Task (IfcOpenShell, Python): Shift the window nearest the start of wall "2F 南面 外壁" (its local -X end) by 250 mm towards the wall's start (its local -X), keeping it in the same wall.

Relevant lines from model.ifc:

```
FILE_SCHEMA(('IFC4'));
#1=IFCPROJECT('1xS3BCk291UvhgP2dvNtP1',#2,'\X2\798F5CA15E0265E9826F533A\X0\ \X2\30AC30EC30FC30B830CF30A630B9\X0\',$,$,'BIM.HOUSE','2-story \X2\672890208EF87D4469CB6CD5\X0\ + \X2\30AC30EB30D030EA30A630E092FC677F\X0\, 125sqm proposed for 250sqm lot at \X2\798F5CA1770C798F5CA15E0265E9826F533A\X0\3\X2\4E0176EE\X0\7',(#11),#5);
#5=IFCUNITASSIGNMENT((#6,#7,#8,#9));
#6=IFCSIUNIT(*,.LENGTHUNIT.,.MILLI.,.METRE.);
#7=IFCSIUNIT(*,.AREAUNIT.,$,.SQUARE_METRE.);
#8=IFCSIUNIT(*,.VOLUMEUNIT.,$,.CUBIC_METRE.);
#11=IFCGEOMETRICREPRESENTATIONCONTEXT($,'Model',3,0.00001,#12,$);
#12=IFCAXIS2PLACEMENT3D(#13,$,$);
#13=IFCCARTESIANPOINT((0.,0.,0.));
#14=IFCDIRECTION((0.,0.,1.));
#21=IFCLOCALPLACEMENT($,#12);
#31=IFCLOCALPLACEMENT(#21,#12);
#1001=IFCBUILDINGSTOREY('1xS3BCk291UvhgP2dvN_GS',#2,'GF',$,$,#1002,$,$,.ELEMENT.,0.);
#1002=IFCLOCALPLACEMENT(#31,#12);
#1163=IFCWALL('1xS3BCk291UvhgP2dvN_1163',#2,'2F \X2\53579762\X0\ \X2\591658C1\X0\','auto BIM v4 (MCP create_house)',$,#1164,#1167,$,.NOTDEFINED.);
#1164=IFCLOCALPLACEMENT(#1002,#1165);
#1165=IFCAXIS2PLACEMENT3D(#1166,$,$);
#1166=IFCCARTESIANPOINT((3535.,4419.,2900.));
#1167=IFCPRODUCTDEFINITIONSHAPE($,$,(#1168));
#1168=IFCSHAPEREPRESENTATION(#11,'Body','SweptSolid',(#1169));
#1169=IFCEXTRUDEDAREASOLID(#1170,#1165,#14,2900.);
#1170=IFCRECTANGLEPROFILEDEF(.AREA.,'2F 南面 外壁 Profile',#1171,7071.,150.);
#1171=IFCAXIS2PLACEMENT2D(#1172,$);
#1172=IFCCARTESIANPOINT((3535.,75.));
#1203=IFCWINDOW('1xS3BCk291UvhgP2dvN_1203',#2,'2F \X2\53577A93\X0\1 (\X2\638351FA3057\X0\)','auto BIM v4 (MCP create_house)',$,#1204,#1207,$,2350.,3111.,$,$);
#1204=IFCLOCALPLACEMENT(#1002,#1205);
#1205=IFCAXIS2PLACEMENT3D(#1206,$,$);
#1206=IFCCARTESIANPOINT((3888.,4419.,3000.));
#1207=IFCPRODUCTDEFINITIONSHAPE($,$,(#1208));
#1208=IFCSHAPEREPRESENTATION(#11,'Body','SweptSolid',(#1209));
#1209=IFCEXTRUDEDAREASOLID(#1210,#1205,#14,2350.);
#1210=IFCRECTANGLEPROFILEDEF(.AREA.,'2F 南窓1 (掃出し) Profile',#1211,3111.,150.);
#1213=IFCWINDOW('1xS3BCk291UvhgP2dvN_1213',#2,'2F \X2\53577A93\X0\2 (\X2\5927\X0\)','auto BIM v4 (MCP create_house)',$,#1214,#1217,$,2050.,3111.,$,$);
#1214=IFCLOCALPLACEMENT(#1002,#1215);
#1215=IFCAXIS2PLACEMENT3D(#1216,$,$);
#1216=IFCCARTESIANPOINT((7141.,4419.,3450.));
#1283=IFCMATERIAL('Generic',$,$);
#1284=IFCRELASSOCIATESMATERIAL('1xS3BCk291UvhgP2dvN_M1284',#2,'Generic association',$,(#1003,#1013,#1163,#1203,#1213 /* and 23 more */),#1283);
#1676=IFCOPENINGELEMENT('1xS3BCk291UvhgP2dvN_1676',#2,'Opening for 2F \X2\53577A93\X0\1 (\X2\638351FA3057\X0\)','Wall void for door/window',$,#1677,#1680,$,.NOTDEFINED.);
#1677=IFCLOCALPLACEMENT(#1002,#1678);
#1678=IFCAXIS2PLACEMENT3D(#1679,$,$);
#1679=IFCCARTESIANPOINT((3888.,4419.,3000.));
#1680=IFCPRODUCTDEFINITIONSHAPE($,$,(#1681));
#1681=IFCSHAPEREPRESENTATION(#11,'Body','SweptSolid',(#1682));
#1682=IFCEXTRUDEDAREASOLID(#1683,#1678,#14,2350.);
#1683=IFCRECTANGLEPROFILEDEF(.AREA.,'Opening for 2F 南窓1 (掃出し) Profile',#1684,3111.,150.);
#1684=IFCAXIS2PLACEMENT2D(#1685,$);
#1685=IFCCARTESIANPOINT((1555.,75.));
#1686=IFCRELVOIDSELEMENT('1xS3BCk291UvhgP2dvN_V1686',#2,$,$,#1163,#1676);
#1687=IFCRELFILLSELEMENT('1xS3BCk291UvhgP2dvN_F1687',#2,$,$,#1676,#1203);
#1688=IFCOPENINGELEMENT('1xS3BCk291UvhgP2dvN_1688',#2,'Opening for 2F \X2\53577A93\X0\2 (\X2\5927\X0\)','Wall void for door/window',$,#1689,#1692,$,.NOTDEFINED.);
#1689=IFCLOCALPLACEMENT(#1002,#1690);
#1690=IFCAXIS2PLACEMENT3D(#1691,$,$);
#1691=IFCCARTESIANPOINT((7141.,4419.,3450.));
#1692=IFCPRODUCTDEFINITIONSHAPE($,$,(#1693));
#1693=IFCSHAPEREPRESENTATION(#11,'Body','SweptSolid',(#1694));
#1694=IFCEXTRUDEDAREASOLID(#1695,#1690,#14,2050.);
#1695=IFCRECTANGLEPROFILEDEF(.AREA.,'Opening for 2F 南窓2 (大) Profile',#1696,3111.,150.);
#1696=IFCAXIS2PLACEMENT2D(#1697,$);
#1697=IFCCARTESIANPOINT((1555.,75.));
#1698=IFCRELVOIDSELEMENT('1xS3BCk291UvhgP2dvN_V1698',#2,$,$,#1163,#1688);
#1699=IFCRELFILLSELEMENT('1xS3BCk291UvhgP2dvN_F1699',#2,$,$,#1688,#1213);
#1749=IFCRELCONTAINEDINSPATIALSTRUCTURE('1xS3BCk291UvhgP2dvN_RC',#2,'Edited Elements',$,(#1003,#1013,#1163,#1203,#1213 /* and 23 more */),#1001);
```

```python
import ifcopenshell
import ifcopenshell.api.geometry
import ifcopenshell.util.placement
import ifcopenshell.util.unit

model = ifcopenshell.open("model.ifc")
unit_scale = ifcopenshell.util.unit.calculate_unit_scale(model)

window = model.by_guid("1xS3BCk291UvhgP2dvN_1203")
opening = window.FillsVoids[0].RelatingOpeningElement
wall = opening.VoidsElements[0].RelatingBuildingElement

wall_matrix = ifcopenshell.util.placement.get_local_placement(wall.ObjectPlacement)
shift = wall_matrix[:3, 0] * -0.25 / unit_scale
before = ifcopenshell.util.placement.get_local_placement(window.ObjectPlacement)[:3, 3].copy()

# The window is not placed relative to its opening, so move both.
for product in (opening, window):
    matrix = ifcopenshell.util.placement.get_local_placement(product.ObjectPlacement)
    matrix[:3, 3] += shift
    ifcopenshell.api.geometry.edit_object_placement(model, product=product, matrix=matrix, is_si=False)

after = ifcopenshell.util.placement.get_local_placement(window.ObjectPlacement)[:3, 3]
print("window moved by", (after - before).round(3) + 0.0)

model.write("model_v2.ifc")
```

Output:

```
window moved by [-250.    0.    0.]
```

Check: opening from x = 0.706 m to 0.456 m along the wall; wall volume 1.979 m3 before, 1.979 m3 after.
